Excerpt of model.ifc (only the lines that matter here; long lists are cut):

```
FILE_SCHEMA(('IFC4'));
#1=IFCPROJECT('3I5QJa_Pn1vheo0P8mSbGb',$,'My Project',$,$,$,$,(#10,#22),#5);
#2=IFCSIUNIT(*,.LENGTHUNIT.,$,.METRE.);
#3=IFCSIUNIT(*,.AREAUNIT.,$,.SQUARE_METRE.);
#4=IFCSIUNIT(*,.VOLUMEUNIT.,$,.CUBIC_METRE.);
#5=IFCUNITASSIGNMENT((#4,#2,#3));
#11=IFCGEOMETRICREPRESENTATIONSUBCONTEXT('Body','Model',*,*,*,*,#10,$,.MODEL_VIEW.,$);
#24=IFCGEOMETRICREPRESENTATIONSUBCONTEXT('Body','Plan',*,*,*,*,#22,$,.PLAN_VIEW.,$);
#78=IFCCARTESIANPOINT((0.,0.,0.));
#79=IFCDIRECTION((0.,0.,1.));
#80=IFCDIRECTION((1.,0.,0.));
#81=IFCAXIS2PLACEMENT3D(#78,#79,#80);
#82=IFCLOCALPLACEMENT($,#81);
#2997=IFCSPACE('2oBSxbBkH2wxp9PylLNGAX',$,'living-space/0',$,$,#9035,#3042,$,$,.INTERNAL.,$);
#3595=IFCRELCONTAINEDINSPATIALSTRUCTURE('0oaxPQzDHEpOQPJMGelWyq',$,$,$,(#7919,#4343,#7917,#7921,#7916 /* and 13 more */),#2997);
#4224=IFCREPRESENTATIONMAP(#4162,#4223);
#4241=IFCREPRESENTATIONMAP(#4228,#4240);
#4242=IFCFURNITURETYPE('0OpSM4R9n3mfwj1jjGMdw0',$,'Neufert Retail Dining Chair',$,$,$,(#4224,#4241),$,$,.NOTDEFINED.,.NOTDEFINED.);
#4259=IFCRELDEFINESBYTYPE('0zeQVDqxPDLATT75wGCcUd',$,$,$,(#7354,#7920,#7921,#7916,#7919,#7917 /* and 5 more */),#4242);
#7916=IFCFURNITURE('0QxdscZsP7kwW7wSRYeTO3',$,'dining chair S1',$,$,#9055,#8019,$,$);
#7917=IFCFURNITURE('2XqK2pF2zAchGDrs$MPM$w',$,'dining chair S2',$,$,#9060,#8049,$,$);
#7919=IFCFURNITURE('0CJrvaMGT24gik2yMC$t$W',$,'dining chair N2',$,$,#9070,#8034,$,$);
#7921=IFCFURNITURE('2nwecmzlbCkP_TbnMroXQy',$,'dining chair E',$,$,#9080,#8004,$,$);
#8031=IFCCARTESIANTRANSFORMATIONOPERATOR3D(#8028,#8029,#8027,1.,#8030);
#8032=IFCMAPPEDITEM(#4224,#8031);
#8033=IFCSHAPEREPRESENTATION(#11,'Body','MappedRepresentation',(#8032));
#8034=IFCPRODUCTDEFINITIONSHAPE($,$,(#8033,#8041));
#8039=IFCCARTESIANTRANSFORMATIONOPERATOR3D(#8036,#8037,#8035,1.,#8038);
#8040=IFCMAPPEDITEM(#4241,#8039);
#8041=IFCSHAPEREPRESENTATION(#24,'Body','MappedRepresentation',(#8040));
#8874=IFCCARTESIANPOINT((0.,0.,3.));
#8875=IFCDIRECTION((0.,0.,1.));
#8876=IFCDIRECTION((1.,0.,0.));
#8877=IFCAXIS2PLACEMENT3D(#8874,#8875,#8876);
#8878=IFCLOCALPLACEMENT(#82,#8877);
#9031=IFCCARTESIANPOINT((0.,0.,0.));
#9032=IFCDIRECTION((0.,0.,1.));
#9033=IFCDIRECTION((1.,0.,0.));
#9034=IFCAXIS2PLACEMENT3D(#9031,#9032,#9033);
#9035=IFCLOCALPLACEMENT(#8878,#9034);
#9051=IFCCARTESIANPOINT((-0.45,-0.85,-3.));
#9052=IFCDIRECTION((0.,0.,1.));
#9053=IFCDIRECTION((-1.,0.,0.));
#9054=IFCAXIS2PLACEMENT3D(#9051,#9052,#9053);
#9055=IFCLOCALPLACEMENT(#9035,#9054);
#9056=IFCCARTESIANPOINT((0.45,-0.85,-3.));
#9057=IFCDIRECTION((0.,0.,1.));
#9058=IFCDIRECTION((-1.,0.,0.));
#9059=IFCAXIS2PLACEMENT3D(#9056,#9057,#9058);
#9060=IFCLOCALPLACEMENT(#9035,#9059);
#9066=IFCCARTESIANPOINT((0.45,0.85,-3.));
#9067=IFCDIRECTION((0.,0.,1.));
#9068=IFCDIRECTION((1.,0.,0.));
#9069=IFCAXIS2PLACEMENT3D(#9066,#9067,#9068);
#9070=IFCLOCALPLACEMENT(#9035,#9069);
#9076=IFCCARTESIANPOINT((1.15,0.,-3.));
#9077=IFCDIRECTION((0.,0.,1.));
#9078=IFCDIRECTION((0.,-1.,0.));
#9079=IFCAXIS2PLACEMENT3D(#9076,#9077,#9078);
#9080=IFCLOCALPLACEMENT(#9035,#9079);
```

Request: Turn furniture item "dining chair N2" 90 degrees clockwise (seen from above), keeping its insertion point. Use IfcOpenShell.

```python
import ifcopenshell
import ifcopenshell.api.geometry
import ifcopenshell.util.placement

model = ifcopenshell.open("model.ifc")

item = model.by_guid("0CJrvaMGT24gik2yMC$t$W")
matrix = ifcopenshell.util.placement.get_local_placement(item.ObjectPlacement)
matrix = matrix @ ifcopenshell.util.placement.rotation(-90, "Z")
ifcopenshell.api.geometry.edit_object_placement(model, product=item, matrix=matrix, is_si=False)

print(ifcopenshell.util.placement.get_local_placement(item.ObjectPlacement).round(3) + 0.0)

model.write("model_rev.ifc")
```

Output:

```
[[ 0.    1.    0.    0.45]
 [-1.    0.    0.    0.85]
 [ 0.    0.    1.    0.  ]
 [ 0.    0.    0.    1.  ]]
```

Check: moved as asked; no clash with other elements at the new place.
